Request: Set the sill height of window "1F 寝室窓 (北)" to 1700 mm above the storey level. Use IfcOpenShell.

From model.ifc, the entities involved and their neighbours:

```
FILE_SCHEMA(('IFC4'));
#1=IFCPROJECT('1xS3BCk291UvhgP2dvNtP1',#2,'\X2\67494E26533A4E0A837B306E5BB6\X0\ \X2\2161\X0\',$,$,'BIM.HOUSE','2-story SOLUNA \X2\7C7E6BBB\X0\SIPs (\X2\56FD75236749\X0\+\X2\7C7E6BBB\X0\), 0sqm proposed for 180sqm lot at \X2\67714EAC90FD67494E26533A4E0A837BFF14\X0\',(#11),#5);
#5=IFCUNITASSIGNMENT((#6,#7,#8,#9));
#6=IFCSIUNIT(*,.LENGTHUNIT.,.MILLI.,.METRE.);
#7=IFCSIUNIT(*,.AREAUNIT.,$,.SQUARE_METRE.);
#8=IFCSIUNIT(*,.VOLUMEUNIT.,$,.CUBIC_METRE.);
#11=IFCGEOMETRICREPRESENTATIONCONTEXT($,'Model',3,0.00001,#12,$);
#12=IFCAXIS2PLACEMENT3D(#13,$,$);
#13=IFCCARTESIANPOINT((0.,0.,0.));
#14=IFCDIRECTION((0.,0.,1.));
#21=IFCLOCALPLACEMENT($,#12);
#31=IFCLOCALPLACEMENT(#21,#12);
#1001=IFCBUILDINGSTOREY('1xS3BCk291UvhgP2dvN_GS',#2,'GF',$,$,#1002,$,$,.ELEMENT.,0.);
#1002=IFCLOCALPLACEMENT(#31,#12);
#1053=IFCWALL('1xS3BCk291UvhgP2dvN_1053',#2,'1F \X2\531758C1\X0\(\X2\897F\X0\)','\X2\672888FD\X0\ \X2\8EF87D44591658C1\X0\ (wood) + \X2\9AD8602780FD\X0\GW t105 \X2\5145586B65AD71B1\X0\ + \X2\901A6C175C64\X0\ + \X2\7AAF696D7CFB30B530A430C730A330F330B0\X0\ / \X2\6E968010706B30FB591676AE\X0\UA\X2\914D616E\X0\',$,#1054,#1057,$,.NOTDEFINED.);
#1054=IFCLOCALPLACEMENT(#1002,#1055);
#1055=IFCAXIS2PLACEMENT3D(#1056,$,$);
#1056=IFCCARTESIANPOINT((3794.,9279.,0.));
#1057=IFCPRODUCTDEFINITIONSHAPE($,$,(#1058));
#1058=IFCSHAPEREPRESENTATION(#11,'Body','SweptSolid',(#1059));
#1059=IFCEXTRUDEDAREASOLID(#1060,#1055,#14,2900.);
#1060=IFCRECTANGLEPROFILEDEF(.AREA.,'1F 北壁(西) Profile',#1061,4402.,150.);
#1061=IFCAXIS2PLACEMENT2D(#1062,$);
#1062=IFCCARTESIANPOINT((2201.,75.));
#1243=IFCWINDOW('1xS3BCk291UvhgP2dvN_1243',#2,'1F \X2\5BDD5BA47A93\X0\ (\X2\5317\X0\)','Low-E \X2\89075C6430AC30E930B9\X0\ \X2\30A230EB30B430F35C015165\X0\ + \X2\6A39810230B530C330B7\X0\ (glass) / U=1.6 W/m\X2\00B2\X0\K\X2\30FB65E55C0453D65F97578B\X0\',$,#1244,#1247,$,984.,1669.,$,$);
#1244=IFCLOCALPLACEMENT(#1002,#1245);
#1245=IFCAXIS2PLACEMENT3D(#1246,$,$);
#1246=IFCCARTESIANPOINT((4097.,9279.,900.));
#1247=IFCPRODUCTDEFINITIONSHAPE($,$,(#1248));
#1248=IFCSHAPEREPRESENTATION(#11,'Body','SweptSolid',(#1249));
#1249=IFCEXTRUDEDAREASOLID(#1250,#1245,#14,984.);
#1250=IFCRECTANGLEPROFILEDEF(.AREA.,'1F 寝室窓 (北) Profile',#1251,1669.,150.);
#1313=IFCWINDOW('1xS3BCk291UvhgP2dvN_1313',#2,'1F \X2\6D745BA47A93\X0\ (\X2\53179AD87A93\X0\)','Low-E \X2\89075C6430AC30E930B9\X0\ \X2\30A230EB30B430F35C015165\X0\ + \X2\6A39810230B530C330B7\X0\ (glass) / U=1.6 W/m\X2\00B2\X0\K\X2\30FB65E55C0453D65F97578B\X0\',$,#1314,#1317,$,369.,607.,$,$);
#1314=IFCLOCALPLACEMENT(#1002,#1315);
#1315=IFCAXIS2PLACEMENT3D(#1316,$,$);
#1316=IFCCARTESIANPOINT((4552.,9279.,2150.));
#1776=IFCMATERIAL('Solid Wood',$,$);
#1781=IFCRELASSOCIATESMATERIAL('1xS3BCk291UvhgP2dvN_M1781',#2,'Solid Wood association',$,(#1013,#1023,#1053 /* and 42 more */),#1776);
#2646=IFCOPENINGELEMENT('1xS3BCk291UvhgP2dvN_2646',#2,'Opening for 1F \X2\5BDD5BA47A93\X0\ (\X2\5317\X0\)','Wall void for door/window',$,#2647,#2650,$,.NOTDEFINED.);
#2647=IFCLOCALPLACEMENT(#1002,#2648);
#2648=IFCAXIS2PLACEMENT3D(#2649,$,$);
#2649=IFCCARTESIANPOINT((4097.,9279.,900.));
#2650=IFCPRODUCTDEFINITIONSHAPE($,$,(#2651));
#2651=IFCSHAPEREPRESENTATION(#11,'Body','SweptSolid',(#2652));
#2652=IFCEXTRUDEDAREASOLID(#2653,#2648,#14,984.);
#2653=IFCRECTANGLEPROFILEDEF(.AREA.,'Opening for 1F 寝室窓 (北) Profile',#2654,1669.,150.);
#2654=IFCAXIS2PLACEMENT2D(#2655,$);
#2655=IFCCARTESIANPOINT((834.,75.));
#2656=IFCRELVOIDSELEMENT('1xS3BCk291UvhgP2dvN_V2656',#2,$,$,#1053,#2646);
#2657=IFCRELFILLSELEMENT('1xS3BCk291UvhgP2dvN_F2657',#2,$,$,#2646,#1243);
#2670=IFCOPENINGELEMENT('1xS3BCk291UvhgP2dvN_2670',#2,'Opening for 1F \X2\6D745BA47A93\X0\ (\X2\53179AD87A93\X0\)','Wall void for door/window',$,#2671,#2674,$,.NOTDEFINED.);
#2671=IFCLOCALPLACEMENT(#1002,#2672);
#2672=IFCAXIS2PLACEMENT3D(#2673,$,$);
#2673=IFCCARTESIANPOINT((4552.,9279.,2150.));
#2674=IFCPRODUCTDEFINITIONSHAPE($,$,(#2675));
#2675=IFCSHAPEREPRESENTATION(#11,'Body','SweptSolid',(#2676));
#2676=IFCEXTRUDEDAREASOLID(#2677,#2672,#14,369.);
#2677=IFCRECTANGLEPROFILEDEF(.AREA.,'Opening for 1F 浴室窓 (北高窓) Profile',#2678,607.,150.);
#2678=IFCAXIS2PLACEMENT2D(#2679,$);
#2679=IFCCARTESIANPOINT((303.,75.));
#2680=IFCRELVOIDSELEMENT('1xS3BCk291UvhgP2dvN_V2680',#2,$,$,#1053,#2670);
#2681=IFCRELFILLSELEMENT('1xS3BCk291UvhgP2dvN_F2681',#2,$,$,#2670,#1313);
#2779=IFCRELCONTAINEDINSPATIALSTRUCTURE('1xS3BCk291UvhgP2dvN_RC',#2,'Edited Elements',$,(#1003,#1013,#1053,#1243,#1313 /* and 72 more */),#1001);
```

```python
import numpy as np
import ifcopenshell
import ifcopenshell.api.geometry
import ifcopenshell.geom
import ifcopenshell.util.element
import ifcopenshell.util.placement
import ifcopenshell.util.shape
import ifcopenshell.util.unit

model = ifcopenshell.open("model.ifc")
unit_scale = ifcopenshell.util.unit.calculate_unit_scale(model)

window = model.by_guid("1xS3BCk291UvhgP2dvN_1243")
opening = window.FillsVoids[0].RelatingOpeningElement
storey = ifcopenshell.util.element.get_container(window, ifc_class="IfcBuildingStorey")
level = ifcopenshell.util.placement.get_local_placement(storey.ObjectPlacement)[2, 3]

# The opening's origin need not be at the sill, so measure its lowest point.
shape = ifcopenshell.geom.create_shape(ifcopenshell.geom.settings(), opening)
bottom = ifcopenshell.util.shape.get_shape_bottom_elevation(shape, shape.geometry) / unit_scale
dz = level + 1700.0 - bottom

shift = np.array([0.0, 0.0, dz])
# The window is not placed relative to its opening, so move both.
for product in (opening, window):
    matrix = ifcopenshell.util.placement.get_local_placement(product.ObjectPlacement)
    matrix[:3, 3] += shift
    ifcopenshell.api.geometry.edit_object_placement(model, product=product, matrix=matrix, is_si=False)

print(f"moved by {dz * unit_scale:+.3f} m")

model.write("model_edited.ifc")
```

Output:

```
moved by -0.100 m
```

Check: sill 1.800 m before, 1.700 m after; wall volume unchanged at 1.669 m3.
